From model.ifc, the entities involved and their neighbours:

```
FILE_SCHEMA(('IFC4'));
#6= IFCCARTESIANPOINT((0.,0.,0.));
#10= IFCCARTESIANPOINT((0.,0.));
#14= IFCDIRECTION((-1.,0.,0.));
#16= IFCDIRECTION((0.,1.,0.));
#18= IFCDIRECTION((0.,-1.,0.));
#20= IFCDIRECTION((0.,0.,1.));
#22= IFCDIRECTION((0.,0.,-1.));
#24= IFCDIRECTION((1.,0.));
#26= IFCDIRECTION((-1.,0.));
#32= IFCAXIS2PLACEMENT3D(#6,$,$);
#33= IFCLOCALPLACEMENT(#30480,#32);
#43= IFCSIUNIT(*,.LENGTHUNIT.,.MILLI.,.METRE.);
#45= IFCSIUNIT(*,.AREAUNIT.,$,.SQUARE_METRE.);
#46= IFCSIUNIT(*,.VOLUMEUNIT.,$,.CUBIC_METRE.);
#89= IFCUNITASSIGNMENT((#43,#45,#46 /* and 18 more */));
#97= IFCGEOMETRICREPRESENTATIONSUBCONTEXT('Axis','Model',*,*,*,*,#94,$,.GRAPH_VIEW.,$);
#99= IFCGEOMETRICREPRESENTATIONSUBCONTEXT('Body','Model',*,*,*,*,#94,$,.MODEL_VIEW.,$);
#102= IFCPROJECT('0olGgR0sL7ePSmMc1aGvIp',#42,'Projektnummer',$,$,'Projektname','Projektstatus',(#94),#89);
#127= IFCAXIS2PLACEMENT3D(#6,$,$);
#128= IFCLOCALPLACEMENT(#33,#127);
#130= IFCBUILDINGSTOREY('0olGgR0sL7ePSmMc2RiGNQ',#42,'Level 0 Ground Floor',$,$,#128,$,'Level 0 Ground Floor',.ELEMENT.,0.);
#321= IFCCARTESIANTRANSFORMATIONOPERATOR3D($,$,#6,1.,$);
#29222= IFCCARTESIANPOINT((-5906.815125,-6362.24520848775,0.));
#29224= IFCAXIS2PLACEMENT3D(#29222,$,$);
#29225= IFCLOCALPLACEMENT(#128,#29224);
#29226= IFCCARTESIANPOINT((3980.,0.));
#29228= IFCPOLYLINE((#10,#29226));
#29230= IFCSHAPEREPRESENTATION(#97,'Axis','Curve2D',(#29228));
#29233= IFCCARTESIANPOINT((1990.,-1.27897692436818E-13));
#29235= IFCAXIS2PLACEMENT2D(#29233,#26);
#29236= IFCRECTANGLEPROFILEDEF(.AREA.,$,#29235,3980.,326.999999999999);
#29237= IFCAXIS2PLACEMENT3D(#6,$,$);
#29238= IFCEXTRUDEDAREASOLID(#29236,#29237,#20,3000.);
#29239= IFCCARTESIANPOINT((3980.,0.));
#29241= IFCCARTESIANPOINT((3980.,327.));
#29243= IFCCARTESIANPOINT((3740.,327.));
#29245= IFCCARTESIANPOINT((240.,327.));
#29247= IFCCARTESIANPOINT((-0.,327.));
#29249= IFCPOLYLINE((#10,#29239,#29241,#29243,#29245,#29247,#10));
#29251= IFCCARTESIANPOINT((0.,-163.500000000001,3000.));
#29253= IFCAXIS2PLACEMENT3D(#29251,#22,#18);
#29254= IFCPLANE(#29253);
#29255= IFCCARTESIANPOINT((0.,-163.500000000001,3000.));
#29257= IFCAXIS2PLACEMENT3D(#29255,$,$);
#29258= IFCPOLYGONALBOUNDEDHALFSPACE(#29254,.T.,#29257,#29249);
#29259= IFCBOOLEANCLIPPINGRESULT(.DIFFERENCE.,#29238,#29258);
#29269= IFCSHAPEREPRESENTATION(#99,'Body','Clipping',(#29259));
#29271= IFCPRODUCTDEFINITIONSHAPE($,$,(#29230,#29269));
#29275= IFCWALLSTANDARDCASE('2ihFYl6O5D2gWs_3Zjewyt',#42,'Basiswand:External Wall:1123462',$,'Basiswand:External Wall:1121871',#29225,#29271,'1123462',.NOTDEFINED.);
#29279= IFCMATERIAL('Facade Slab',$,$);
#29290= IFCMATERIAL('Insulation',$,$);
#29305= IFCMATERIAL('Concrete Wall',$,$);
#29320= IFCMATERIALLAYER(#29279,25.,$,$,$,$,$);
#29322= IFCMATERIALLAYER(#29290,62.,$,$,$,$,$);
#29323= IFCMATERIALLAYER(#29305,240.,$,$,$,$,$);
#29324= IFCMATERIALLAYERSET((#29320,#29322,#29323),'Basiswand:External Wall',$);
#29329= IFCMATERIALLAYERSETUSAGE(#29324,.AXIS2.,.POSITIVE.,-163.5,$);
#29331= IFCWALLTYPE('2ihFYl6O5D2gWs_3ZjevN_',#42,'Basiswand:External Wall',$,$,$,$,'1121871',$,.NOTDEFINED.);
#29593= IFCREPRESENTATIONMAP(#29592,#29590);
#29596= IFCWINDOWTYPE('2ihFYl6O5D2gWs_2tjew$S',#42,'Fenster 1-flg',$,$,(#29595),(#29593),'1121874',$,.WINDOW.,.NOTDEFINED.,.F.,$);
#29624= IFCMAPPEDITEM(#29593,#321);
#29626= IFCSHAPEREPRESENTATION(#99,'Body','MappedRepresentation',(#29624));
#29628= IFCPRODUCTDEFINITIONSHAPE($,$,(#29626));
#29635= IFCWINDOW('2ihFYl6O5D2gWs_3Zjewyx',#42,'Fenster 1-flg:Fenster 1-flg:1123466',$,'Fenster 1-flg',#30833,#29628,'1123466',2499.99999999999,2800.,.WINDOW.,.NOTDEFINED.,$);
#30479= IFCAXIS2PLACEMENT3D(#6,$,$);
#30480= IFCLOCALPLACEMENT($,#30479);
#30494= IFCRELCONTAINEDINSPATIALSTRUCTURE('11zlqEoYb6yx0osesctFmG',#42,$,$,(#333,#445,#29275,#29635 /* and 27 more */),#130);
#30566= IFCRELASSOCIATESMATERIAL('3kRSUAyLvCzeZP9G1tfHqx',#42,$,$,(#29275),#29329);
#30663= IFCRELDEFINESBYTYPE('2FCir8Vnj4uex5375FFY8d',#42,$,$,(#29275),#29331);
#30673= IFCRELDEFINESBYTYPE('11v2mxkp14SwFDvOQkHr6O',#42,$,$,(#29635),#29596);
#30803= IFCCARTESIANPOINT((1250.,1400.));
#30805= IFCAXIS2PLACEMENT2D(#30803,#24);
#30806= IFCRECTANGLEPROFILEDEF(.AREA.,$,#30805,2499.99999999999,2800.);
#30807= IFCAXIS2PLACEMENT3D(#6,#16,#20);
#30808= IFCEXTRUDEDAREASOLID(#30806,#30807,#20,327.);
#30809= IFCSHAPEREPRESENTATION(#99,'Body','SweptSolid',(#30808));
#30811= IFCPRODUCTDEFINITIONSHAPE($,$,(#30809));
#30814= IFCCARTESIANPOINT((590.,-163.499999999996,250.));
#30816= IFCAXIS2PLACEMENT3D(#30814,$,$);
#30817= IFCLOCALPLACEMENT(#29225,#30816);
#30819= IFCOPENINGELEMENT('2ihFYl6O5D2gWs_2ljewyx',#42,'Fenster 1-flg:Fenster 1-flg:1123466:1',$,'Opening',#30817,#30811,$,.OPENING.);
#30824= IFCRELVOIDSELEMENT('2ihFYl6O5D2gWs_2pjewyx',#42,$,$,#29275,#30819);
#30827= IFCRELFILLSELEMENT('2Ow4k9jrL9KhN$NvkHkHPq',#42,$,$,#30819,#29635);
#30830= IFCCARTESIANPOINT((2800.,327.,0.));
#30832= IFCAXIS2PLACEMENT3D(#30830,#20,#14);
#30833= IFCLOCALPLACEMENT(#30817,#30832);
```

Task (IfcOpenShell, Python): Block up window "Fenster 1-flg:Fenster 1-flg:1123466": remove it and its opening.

```python
import ifcopenshell
import ifcopenshell.api.feature
import ifcopenshell.api.root
import ifcopenshell.geom
import ifcopenshell.util.shape

model = ifcopenshell.open("model.ifc")
settings = ifcopenshell.geom.settings()


def volume(element):
    """Net volume in cubic metres, openings subtracted."""
    shape = ifcopenshell.geom.create_shape(settings, element)
    return ifcopenshell.util.shape.get_volume(shape.geometry)


window = model.by_id(29635)
opening = window.FillsVoids[0].RelatingOpeningElement
wall = opening.VoidsElements[0].RelatingBuildingElement
before = volume(wall)

ifcopenshell.api.root.remove_product(model, product=window)
ifcopenshell.api.feature.remove_feature(model, feature=opening)

after = volume(wall)

print(f"wall volume {before:.3f} -> {after:.3f} m3")

model.write("model_updated.ifc")
```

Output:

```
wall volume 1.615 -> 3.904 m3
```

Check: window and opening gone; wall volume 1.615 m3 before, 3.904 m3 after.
